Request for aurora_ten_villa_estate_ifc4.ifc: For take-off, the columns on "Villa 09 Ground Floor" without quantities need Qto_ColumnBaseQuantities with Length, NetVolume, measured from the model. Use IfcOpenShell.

First a look at what the model holds.

```python
import ifcopenshell
import ifcopenshell.util.element
import ifcopenshell.util.unit

model = ifcopenshell.open("aurora_ten_villa_estate_ifc4.ifc")
print(model.schema)
for unit_type in ("LENGTHUNIT", "AREAUNIT", "VOLUMEUNIT"):
    print(unit_type, ifcopenshell.util.unit.calculate_unit_scale(model, unit_type))
storey = next(s for s in model.by_type("IfcBuildingStorey") if s.Name == "Villa 09 Ground Floor")
columns = [e for e in ifcopenshell.util.element.get_decomposition(storey) if e.is_a("IfcColumn")]
for e in sorted(columns, key=lambda e: e.id()):
    print(e.id(), e.is_a(), e.Name, list(ifcopenshell.util.element.get_psets(e, qtos_only=True)), sep=" | ")
```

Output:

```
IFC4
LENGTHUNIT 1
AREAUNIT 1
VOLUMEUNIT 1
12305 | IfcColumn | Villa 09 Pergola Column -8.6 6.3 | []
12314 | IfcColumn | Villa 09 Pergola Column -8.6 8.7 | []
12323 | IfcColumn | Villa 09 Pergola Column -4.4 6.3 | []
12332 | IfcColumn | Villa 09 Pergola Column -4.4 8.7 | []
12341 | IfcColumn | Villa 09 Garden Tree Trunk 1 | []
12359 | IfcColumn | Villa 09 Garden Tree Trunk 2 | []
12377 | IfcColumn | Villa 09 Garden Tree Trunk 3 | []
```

```python
import ifcopenshell
import ifcopenshell.api.pset
import ifcopenshell.geom
import ifcopenshell.util.element
import ifcopenshell.util.shape
import ifcopenshell.util.unit

model = ifcopenshell.open("aurora_ten_villa_estate_ifc4.ifc")
unit_scale = ifcopenshell.util.unit.calculate_unit_scale(model)
volume_scale = ifcopenshell.util.unit.calculate_unit_scale(model, "VOLUMEUNIT")
settings = ifcopenshell.geom.settings()

storey = next(s for s in model.by_type("IfcBuildingStorey") if s.Name == "Villa 09 Ground Floor")
columns = [e for e in ifcopenshell.util.element.get_decomposition(storey) if e.is_a("IfcColumn")]

for e in sorted(columns, key=lambda e: e.id()):
    if ifcopenshell.util.element.get_psets(e, qtos_only=True, should_inherit=False):
        continue
    # Geometry comes back in metres, in the element's own axes.
    shape = ifcopenshell.geom.create_shape(settings, e)
    values = {
        "Length": ifcopenshell.util.shape.get_z(shape.geometry) / unit_scale,
        "NetVolume": ifcopenshell.util.shape.get_volume(shape.geometry) / volume_scale,
    }
    qto = ifcopenshell.api.pset.add_qto(model, product=e, name="Qto_ColumnBaseQuantities")
    ifcopenshell.api.pset.edit_qto(model, qto=qto, properties=values)
    print(e.id(), {k: round(v, 3) for k, v in values.items()})

model.write("aurora_ten_villa_estate_ifc4-out.ifc")
```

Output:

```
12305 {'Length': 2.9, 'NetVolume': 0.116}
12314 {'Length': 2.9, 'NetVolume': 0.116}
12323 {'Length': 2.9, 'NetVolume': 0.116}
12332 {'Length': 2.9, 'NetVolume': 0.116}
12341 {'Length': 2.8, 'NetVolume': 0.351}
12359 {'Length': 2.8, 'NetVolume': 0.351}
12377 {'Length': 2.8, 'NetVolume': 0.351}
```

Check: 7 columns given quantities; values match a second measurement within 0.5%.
